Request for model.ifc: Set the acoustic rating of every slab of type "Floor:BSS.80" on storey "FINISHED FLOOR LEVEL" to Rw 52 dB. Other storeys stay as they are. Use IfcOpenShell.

First a look at what the model holds.

```python
import ifcopenshell
import ifcopenshell.util.element

model = ifcopenshell.open("model.ifc")
print(model.schema)
storey = next(s for s in model.by_type("IfcBuildingStorey") if s.Name == "FINISHED FLOOR LEVEL")
slabs = [e for e in ifcopenshell.util.element.get_decomposition(storey) if e.is_a("IfcSlab")]
seen = {}
for e in slabs:
    element_type = ifcopenshell.util.element.get_type(e)
    key = (element_type.Name if element_type != e and element_type else None, ifcopenshell.util.element.get_pset(e, "Pset_SlabCommon", "AcousticRating"))
    seen[key] = seen.get(key, 0) + 1
for (name, value), count in sorted(seen.items(), key=str):
    print(count, "x", name, "|", value)
```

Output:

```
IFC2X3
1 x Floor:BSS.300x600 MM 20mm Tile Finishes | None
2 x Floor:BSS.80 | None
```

```python
import ifcopenshell
import ifcopenshell.api.pset
import ifcopenshell.util.element

model = ifcopenshell.open("model.ifc")

storey = next(s for s in model.by_type("IfcBuildingStorey") if s.Name == "FINISHED FLOOR LEVEL")
slabs = [e for e in ifcopenshell.util.element.get_decomposition(storey) if e.is_a("IfcSlab")]

count = 0
for e in slabs:
    element_type = ifcopenshell.util.element.get_type(e)
    if element_type in (None, e) or element_type.Name != "Floor:BSS.80":
        continue
    # add_pset returns the element's existing set when there is one.
    pset = ifcopenshell.api.pset.add_pset(model, product=e, name="Pset_SlabCommon")
    ifcopenshell.api.pset.edit_pset(model, pset=pset, properties={"AcousticRating": "Rw 52 dB"})
    count += 1

print(count, "slabs updated")

model.write("model-out.ifc")
```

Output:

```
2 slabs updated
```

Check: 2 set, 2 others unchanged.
